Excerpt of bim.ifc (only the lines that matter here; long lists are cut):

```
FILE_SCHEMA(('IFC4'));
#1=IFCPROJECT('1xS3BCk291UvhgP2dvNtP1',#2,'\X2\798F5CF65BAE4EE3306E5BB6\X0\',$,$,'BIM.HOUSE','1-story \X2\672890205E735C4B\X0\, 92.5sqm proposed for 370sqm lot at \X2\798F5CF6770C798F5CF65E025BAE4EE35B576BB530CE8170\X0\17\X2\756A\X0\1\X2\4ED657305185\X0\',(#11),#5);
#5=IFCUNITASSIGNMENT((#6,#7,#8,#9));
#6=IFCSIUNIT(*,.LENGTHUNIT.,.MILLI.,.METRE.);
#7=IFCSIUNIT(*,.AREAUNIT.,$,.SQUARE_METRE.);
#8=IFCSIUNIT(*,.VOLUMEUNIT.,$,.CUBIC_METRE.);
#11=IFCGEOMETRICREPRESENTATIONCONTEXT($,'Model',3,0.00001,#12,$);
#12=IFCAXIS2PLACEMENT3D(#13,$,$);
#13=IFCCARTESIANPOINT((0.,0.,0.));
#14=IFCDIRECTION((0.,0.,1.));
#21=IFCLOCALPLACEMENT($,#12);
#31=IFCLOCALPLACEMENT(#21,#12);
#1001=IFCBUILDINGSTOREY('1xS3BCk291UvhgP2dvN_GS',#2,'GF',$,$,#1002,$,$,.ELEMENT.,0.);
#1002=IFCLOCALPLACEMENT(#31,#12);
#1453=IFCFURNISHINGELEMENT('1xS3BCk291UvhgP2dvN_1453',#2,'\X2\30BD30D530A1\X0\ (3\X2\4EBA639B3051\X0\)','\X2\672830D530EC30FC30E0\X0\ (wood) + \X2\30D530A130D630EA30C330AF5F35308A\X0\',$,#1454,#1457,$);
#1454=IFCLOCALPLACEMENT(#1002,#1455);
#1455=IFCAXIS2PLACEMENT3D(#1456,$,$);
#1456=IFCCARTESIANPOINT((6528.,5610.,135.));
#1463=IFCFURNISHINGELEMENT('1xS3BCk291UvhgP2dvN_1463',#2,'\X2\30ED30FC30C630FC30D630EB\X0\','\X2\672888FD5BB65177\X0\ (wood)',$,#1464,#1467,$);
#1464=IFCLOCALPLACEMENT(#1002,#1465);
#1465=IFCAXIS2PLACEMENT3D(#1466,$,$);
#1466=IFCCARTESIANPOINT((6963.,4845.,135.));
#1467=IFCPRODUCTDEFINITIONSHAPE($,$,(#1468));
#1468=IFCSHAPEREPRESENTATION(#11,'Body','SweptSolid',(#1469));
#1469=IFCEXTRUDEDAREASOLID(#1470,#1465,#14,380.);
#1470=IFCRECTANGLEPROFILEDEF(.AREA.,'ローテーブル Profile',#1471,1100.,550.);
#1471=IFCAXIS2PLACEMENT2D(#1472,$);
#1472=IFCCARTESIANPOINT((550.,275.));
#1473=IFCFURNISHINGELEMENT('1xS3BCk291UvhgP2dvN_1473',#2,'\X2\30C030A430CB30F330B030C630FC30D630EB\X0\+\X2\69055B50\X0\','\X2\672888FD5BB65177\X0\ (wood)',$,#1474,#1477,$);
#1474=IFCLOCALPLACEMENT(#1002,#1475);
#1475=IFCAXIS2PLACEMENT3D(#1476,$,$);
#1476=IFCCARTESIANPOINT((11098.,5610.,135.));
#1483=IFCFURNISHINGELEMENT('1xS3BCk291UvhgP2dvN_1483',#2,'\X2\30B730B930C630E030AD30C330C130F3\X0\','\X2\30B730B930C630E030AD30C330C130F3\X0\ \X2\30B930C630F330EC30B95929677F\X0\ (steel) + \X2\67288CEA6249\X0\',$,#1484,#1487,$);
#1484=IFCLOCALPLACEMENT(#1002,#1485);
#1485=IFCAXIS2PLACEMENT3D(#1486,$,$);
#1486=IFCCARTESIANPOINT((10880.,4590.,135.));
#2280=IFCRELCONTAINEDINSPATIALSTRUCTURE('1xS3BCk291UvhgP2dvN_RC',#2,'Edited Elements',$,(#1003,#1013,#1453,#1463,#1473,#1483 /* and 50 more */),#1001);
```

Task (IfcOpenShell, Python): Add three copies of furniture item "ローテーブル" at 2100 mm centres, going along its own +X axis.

```python
import ifcopenshell
import ifcopenshell.api.geometry
import ifcopenshell.api.root
import ifcopenshell.util.element
import ifcopenshell.util.placement
import ifcopenshell.util.unit

model = ifcopenshell.open("bim.ifc")
unit_scale = ifcopenshell.util.unit.calculate_unit_scale(model)


def reuse_history(source, copy):
    """copy_class also copies each property set's owner history, people and application; keep the originals."""
    for rel in copy.IsDefinedBy:
        if rel.is_a("IfcRelDefinesByProperties") and (history := rel.RelatingPropertyDefinition.OwnerHistory):
            rel.RelatingPropertyDefinition.OwnerHistory = source.OwnerHistory
            ifcopenshell.util.element.remove_deep2(model, history)


source = model.by_id(1463)
base = ifcopenshell.util.placement.get_local_placement(source.ObjectPlacement)
step = base[:3, 0] * 2.1 / unit_scale

for i in range(1, 4):
    copy = ifcopenshell.api.root.copy_class(model, product=source)
    copy.Representation = ifcopenshell.util.element.copy_deep(
        model, source.Representation, exclude=["IfcGeometricRepresentationContext", "IfcRepresentationMap"]
    )
    reuse_history(source, copy)
    matrix = base.copy()
    matrix[:3, 3] += i * step
    print("added at", matrix[:3, 3].round(3) + 0.0)
    ifcopenshell.api.geometry.edit_object_placement(model, product=copy, matrix=matrix, is_si=False)

model.write("bim-out.ifc")
```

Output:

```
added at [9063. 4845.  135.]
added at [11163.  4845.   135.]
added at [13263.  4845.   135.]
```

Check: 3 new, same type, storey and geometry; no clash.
